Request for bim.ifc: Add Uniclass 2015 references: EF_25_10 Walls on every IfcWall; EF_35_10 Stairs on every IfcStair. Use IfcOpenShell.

First a look at what the model holds.

```python
import ifcopenshell

model = ifcopenshell.open("bim.ifc")
print(model.schema)
print("classifications:", [c.Name for c in model.by_type("IfcClassification")])
for ifc_class in ("IfcDoor", "IfcRoof", "IfcStair", "IfcWall", "IfcWindow"):
    print(ifc_class, len(model.by_type(ifc_class)))
```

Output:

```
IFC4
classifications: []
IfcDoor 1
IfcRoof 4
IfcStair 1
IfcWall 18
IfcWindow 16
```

```python
import ifcopenshell
import ifcopenshell.api.classification

model = ifcopenshell.open("bim.ifc")

system = ifcopenshell.api.classification.add_classification(model, classification="Uniclass 2015")

codes = {
    "IfcWall": ("EF_25_10", "Walls"),
    "IfcStair": ("EF_35_10", "Stairs"),
}
for ifc_class, (code, name) in codes.items():
    products = model.by_type(ifc_class)
    ifcopenshell.api.classification.add_reference(
        model, products=products, classification=system, identification=code, name=name
    )
    print(code, len(products))

model.write("bim-out.ifc")
```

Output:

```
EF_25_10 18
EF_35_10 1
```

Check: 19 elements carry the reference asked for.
